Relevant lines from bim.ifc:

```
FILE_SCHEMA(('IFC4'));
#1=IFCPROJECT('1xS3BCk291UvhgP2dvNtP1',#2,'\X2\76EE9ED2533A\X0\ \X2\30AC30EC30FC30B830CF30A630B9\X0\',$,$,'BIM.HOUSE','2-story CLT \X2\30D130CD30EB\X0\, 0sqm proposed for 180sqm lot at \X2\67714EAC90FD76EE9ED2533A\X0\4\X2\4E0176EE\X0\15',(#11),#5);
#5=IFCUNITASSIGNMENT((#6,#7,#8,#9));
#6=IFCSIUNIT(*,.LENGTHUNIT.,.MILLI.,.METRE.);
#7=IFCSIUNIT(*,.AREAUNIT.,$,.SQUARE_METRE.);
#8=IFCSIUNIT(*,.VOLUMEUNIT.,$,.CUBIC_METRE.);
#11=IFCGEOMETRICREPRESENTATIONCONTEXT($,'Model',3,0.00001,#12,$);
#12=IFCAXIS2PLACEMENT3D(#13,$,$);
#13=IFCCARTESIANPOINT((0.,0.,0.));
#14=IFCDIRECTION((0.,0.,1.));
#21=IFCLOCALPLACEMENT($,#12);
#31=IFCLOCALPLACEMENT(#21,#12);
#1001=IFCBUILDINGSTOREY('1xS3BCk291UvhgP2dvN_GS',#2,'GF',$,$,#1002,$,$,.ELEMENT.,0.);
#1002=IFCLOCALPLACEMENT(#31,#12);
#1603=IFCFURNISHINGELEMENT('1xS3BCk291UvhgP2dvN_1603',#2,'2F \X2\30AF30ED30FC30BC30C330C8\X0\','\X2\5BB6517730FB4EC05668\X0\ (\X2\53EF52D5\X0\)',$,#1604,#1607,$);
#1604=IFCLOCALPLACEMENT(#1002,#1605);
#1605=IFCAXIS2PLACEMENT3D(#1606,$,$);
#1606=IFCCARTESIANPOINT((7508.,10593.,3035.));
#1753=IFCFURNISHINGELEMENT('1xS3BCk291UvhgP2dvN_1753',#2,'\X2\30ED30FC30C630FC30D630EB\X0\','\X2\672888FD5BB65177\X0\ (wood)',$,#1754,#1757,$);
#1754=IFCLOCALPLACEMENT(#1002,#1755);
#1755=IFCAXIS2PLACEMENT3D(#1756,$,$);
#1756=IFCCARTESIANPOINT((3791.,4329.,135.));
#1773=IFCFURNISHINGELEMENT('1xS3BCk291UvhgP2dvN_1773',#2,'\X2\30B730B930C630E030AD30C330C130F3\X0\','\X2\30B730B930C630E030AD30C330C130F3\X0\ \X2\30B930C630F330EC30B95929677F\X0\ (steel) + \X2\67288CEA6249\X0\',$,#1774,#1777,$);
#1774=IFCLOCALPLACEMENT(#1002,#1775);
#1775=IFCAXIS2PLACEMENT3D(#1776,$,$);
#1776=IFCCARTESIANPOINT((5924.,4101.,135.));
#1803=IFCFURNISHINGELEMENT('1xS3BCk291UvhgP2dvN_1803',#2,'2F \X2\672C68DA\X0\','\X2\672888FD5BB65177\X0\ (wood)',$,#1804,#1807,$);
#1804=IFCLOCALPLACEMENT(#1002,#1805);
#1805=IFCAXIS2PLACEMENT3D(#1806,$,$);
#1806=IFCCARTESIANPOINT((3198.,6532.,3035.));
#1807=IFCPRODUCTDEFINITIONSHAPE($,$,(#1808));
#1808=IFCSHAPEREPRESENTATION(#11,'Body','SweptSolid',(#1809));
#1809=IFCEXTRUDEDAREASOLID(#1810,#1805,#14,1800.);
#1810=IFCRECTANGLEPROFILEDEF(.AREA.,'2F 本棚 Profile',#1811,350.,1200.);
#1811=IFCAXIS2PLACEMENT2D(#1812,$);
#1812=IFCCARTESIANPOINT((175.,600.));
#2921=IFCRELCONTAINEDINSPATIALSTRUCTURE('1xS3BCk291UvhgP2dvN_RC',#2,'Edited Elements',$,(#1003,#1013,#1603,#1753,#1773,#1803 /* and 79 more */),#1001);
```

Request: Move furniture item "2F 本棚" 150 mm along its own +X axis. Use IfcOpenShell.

```python
import ifcopenshell
import ifcopenshell.api.geometry
import ifcopenshell.util.placement

model = ifcopenshell.open("bim.ifc")

item = model.by_id(1803)
matrix = ifcopenshell.util.placement.get_local_placement(item.ObjectPlacement)
matrix[:3, 3] += matrix[:3, 0] * 150.0
ifcopenshell.api.geometry.edit_object_placement(model, product=item, matrix=matrix, is_si=False)

print(ifcopenshell.util.placement.get_local_placement(item.ObjectPlacement).round(3) + 0.0)

model.write("bim_v2.ifc")
```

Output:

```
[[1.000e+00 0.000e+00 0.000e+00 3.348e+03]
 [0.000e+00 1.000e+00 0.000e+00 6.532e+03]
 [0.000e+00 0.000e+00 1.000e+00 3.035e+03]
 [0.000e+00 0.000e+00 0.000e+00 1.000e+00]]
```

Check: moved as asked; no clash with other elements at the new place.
